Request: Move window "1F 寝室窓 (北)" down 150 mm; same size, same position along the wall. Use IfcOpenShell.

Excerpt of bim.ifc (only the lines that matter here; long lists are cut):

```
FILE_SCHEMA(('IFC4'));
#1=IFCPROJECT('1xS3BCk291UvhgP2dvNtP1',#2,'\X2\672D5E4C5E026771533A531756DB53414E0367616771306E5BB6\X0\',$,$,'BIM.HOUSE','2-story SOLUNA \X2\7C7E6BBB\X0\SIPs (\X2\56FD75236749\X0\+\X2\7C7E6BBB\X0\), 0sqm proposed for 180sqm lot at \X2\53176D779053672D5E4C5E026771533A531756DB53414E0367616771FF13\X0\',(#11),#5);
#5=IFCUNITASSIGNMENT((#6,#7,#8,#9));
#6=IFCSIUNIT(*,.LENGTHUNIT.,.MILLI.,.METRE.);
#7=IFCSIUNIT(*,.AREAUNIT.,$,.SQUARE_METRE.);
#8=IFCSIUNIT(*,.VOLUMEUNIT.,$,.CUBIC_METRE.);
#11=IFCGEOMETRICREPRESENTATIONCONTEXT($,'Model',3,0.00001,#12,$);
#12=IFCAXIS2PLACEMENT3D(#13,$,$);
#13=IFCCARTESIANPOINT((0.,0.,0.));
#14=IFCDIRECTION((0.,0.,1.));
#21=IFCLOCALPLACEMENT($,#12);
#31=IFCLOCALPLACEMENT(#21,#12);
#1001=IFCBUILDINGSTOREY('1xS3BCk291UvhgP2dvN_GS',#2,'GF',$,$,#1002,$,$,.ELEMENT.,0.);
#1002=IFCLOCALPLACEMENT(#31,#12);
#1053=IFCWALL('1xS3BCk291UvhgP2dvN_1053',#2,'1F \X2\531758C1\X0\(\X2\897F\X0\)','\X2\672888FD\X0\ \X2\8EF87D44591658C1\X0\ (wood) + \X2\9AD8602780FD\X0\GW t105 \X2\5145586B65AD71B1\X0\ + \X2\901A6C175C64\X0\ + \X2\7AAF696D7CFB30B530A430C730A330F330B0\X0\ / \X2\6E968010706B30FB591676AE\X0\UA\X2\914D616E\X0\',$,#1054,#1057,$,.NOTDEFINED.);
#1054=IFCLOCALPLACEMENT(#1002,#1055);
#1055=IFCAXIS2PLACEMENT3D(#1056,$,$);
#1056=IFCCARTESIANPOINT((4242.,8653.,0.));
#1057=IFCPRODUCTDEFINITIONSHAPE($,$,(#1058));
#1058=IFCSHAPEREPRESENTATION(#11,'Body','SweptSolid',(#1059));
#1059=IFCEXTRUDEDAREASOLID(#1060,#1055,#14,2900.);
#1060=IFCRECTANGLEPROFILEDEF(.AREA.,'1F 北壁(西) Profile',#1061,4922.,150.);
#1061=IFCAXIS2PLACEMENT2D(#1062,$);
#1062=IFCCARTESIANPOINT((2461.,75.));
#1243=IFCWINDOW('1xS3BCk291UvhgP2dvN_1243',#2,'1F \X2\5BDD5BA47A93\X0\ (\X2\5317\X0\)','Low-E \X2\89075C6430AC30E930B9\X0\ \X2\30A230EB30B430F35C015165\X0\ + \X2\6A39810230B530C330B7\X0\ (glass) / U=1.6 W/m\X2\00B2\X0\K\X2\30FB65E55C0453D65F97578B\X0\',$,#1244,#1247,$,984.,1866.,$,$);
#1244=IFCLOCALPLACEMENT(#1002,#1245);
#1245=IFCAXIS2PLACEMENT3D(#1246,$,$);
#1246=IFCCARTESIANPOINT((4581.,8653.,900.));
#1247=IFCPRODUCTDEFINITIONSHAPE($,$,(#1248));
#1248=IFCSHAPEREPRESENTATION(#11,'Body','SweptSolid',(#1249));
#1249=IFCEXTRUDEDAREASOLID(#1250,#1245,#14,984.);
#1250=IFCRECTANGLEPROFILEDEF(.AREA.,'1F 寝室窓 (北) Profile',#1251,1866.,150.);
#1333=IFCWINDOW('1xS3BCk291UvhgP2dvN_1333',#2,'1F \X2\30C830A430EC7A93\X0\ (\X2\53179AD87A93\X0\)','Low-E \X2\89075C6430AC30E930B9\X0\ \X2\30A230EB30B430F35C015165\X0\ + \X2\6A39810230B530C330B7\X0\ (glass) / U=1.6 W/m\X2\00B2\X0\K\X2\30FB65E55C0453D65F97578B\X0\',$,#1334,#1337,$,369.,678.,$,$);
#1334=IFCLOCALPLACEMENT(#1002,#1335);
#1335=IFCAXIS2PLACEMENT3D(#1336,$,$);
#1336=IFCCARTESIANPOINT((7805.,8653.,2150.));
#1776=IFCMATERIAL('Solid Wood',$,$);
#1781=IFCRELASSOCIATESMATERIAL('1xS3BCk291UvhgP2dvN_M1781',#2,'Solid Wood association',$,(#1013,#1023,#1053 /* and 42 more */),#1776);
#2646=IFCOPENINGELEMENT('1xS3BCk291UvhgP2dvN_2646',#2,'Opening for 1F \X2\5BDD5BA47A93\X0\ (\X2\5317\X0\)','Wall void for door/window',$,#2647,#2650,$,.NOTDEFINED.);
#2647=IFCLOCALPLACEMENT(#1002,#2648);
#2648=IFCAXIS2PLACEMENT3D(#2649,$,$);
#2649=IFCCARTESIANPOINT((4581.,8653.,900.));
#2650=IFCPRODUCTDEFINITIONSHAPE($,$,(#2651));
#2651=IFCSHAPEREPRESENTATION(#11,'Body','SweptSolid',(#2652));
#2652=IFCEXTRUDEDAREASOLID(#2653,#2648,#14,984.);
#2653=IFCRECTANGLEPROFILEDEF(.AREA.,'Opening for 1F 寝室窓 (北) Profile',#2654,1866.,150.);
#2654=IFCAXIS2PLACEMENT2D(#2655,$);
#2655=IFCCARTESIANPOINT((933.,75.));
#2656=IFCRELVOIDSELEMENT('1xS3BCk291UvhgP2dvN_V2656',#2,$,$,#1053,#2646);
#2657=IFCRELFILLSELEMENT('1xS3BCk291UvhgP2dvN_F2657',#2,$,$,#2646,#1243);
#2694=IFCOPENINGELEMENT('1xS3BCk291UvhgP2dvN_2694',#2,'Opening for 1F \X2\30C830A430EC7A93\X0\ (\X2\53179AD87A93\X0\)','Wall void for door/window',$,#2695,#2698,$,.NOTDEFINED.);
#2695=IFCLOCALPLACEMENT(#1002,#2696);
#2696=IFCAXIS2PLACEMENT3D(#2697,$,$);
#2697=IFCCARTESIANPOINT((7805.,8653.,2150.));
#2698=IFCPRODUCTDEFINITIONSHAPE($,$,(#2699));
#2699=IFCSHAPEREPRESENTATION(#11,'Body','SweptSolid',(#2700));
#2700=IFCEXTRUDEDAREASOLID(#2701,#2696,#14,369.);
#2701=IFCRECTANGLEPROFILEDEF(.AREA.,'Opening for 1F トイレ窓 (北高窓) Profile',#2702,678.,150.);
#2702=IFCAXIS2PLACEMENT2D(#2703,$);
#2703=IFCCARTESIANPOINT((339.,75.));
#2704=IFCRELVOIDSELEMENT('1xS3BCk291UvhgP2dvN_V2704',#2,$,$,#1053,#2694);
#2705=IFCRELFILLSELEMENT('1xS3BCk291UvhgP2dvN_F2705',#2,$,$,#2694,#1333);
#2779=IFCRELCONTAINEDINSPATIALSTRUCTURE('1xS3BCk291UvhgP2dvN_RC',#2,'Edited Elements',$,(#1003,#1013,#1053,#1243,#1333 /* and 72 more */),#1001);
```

```python
import numpy as np
import ifcopenshell
import ifcopenshell.api.geometry
import ifcopenshell.util.placement
import ifcopenshell.util.unit

model = ifcopenshell.open("bim.ifc")
unit_scale = ifcopenshell.util.unit.calculate_unit_scale(model)

window = model.by_id(1243)
opening = window.FillsVoids[0].RelatingOpeningElement
dz = -0.15 / unit_scale

shift = np.array([0.0, 0.0, dz])
# The window is not placed relative to its opening, so move both.
for product in (opening, window):
    matrix = ifcopenshell.util.placement.get_local_placement(product.ObjectPlacement)
    matrix[:3, 3] += shift
    ifcopenshell.api.geometry.edit_object_placement(model, product=product, matrix=matrix, is_si=False)

print(f"moved by {dz * unit_scale:+.3f} m")

model.write("bim_rev.ifc")
```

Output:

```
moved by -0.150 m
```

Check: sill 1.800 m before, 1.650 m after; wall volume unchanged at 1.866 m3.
